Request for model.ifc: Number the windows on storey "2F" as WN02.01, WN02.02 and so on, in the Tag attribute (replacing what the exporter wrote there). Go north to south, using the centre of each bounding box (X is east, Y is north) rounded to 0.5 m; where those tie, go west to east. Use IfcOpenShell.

First a look at what the model holds.

```python
import ifcopenshell
import ifcopenshell.util.element
import ifcopenshell.util.placement

model = ifcopenshell.open("model.ifc")
print(model.schema)
storey = next(s for s in model.by_type("IfcBuildingStorey") if s.Name == "2F")
windows = [e for e in ifcopenshell.util.element.get_decomposition(storey) if e.is_a("IfcWindow")]
for e in sorted(windows, key=lambda e: e.id()):
    origin = ifcopenshell.util.placement.get_local_placement(e.ObjectPlacement)[:3, 3]
    print(e.id(), e.Tag, e.Name, origin.round(2) + 0.0, sep=" | ")
```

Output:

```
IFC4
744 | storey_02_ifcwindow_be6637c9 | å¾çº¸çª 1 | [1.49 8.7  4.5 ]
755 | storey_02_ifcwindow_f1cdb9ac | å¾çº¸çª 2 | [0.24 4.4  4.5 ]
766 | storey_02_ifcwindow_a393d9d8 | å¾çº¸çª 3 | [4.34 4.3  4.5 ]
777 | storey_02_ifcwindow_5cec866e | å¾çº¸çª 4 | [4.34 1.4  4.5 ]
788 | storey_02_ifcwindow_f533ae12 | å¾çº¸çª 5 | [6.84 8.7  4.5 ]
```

```python
import ifcopenshell
import ifcopenshell.geom
import ifcopenshell.util.element
import ifcopenshell.util.shape

model = ifcopenshell.open("model.ifc")
settings = ifcopenshell.geom.settings()
settings.set("use-world-coords", True)


def centre(element):
    shape = ifcopenshell.geom.create_shape(settings, element)
    return ifcopenshell.util.shape.get_bbox_centroid(shape.geometry)


storey = next(s for s in model.by_type("IfcBuildingStorey") if s.Name == "2F")
windows = [e for e in ifcopenshell.util.element.get_decomposition(storey) if e.is_a("IfcWindow")]

# Insertion points can sit at a corner or the storey origin, so sort by the geometry (in metres).
centres = {e: centre(e) for e in windows}
windows.sort(key=lambda e: (-round(centres[e][1] / 0.5), centres[e][0]))

for i, e in enumerate(windows, start=1):
    number = f"WN02.{i:02d}"
    e.Tag = number
    print(e.id(), number)

model.write("model_v2.ifc")
```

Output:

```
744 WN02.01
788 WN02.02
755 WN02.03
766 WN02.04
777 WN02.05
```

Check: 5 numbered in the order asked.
